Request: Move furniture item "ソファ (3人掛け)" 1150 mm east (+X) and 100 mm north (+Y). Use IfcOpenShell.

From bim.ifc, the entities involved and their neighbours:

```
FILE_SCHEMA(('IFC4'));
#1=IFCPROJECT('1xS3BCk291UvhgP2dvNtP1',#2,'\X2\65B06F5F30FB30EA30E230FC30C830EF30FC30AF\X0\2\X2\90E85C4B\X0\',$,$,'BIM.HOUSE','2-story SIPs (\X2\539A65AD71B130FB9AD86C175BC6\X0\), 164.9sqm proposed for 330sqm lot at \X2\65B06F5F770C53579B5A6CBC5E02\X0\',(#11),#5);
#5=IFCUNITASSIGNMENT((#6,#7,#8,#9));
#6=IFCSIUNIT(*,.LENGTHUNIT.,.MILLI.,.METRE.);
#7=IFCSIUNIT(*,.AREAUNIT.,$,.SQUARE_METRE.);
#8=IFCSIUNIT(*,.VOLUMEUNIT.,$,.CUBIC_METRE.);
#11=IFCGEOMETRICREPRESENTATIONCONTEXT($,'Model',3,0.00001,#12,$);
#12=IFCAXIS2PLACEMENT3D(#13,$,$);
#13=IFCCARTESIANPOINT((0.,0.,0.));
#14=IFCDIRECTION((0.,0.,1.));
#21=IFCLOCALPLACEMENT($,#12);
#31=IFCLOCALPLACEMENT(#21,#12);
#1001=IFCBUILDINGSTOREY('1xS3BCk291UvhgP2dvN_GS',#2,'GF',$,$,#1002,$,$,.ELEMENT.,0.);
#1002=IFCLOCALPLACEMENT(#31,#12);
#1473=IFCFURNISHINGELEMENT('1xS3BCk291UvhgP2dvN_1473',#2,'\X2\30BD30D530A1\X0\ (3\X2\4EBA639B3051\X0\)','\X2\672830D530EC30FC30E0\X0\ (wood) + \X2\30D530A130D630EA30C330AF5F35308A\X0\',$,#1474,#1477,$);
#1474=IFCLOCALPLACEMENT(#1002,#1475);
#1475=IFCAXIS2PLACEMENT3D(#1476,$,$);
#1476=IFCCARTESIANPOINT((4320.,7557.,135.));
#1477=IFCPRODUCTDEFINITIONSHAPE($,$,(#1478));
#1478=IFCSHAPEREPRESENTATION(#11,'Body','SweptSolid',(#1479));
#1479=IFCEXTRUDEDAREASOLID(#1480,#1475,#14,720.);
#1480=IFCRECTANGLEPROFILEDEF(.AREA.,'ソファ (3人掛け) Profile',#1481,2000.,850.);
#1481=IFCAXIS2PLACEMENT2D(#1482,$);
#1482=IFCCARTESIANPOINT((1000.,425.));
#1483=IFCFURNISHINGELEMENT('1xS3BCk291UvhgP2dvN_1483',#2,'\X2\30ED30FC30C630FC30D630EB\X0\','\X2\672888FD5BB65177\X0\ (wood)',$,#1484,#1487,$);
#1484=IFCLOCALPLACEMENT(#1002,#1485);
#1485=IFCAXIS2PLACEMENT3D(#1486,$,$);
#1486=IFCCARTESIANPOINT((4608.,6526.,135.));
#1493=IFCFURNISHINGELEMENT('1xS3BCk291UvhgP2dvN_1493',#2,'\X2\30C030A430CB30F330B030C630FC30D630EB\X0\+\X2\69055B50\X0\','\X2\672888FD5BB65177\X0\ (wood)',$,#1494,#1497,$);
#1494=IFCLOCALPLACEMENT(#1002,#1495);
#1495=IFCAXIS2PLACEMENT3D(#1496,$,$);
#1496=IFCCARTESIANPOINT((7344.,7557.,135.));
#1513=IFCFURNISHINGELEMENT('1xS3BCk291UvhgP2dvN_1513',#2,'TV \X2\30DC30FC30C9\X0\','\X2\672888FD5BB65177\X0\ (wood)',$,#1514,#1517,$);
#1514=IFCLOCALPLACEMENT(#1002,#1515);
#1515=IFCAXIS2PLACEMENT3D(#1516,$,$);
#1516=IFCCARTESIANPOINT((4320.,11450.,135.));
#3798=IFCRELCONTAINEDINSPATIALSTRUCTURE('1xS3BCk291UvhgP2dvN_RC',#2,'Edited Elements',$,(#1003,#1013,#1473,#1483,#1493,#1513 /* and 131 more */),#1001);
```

```python
import ifcopenshell
import ifcopenshell.api.geometry
import ifcopenshell.util.placement
import ifcopenshell.util.unit

model = ifcopenshell.open("bim.ifc")
unit_scale = ifcopenshell.util.unit.calculate_unit_scale(model)

item = model.by_id(1473)
matrix = ifcopenshell.util.placement.get_local_placement(item.ObjectPlacement)
matrix[0, 3] += 1.15 / unit_scale
matrix[1, 3] += 0.1 / unit_scale
ifcopenshell.api.geometry.edit_object_placement(model, product=item, matrix=matrix, is_si=False)

print(ifcopenshell.util.placement.get_local_placement(item.ObjectPlacement).round(3) + 0.0)

model.write("bim_rev.ifc")
```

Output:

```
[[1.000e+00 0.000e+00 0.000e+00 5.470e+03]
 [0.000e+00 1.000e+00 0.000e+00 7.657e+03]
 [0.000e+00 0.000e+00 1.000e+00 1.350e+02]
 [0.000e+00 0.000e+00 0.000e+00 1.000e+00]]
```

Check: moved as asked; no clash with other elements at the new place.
